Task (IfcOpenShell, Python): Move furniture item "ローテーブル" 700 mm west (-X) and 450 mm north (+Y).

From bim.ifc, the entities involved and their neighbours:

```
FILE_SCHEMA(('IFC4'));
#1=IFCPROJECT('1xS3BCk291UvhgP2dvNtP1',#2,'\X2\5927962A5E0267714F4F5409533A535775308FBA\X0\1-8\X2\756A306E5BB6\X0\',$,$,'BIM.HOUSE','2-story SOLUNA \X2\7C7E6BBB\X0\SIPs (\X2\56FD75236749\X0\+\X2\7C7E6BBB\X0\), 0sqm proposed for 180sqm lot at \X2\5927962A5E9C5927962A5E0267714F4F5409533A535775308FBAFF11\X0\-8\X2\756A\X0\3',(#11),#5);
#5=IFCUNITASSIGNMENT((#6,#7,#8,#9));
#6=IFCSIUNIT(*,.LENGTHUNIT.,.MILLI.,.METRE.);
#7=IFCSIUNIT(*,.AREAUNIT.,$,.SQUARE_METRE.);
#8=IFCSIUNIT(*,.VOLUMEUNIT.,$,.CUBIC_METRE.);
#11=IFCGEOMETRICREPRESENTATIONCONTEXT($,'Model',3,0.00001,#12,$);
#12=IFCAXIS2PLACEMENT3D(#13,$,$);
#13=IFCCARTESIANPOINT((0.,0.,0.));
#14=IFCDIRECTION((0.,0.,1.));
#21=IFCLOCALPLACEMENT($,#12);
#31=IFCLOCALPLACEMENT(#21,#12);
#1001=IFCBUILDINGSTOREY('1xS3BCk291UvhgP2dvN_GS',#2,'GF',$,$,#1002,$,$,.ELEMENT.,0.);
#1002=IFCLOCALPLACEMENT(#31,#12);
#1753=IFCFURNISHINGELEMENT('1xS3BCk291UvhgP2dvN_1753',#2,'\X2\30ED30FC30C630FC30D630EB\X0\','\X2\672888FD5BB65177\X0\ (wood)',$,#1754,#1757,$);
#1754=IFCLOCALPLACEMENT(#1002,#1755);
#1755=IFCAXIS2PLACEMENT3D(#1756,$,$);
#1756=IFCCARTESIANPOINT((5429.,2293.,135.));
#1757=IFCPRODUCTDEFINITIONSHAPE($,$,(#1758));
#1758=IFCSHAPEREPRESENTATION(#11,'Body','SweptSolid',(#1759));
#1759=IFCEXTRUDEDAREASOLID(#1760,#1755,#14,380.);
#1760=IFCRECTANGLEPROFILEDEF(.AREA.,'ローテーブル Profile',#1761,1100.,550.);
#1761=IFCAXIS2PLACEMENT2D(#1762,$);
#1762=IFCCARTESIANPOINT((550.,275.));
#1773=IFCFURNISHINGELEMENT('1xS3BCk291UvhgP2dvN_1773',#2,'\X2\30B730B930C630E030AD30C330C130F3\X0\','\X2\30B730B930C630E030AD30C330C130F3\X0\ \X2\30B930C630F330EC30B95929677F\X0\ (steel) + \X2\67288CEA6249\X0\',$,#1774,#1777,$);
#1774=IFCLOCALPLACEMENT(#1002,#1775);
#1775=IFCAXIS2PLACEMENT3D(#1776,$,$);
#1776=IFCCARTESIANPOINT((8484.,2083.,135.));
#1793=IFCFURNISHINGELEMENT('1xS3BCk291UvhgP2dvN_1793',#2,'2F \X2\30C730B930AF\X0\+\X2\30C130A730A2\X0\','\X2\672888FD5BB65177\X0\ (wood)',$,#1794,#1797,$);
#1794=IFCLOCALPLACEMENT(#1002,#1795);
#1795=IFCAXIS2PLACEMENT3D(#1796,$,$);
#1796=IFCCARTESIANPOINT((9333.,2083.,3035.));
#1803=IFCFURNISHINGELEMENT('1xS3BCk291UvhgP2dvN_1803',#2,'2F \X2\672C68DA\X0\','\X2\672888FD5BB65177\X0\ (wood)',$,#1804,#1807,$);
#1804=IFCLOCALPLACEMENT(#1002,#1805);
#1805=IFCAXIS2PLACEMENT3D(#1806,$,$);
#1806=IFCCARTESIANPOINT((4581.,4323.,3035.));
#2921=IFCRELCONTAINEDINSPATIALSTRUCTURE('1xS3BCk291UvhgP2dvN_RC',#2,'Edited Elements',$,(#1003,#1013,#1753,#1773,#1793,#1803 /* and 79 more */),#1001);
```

```python
import ifcopenshell
import ifcopenshell.api.geometry
import ifcopenshell.util.placement
import ifcopenshell.util.unit

model = ifcopenshell.open("bim.ifc")
unit_scale = ifcopenshell.util.unit.calculate_unit_scale(model)

item = model.by_guid("1xS3BCk291UvhgP2dvN_1753")
matrix = ifcopenshell.util.placement.get_local_placement(item.ObjectPlacement)
matrix[0, 3] -= 0.7 / unit_scale
matrix[1, 3] += 0.45 / unit_scale
ifcopenshell.api.geometry.edit_object_placement(model, product=item, matrix=matrix, is_si=False)

print(ifcopenshell.util.placement.get_local_placement(item.ObjectPlacement).round(3) + 0.0)

model.write("bim-out.ifc")
```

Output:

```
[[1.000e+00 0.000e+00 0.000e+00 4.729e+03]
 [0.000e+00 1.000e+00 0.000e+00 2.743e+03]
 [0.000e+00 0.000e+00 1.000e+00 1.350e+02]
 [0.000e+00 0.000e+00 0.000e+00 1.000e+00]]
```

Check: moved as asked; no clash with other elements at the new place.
